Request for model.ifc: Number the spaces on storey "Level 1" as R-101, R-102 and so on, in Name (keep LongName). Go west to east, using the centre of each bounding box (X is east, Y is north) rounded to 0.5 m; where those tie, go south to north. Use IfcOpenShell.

First a look at what the model holds.

```python
import ifcopenshell
import ifcopenshell.util.element
import ifcopenshell.util.placement

model = ifcopenshell.open("model.ifc")
print(model.schema)
storey = next(s for s in model.by_type("IfcBuildingStorey") if s.Name == "Level 1")
spaces = [e for e in ifcopenshell.util.element.get_decomposition(storey) if e.is_a("IfcSpace")]
for e in sorted(spaces, key=lambda e: e.id()):
    origin = ifcopenshell.util.placement.get_local_placement(e.ObjectPlacement)[:3, 3]
    print(e.id(), e.Name, e.LongName, origin.round(2) + 0.0, sep=" | ")
```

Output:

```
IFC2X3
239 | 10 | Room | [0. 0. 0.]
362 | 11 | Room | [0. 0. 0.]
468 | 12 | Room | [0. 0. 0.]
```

```python
import ifcopenshell
import ifcopenshell.geom
import ifcopenshell.util.element
import ifcopenshell.util.shape

model = ifcopenshell.open("model.ifc")
settings = ifcopenshell.geom.settings()
settings.set("use-world-coords", True)


def centre(element):
    shape = ifcopenshell.geom.create_shape(settings, element)
    return ifcopenshell.util.shape.get_bbox_centroid(shape.geometry)


storey = next(s for s in model.by_type("IfcBuildingStorey") if s.Name == "Level 1")
spaces = [e for e in ifcopenshell.util.element.get_decomposition(storey) if e.is_a("IfcSpace")]

# Insertion points can sit at a corner or the storey origin, so sort by the geometry (in metres).
centres = {e: centre(e) for e in spaces}
spaces.sort(key=lambda e: (round(centres[e][0] / 0.5), centres[e][1]))

for i, e in enumerate(spaces, start=1):
    number = f"R-1{i:02d}"
    e.Name = number
    print(e.id(), number)

model.write("model_v2.ifc")
```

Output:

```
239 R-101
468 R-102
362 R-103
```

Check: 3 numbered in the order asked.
